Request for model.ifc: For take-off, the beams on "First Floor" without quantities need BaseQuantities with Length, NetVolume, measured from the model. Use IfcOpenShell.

First a look at what the model holds.

```python
import ifcopenshell
import ifcopenshell.util.element
import ifcopenshell.util.unit

model = ifcopenshell.open("model.ifc")
print(model.schema)
for unit_type in ("LENGTHUNIT", "AREAUNIT", "VOLUMEUNIT"):
    print(unit_type, ifcopenshell.util.unit.calculate_unit_scale(model, unit_type))
storey = next(s for s in model.by_type("IfcBuildingStorey") if s.Name == "First Floor")
beams = [e for e in ifcopenshell.util.element.get_decomposition(storey) if e.is_a("IfcBeam")]
for e in sorted(beams, key=lambda e: e.id()):
    print(e.id(), e.is_a(), e.Name, list(ifcopenshell.util.element.get_psets(e, qtos_only=True)), sep=" | ")
```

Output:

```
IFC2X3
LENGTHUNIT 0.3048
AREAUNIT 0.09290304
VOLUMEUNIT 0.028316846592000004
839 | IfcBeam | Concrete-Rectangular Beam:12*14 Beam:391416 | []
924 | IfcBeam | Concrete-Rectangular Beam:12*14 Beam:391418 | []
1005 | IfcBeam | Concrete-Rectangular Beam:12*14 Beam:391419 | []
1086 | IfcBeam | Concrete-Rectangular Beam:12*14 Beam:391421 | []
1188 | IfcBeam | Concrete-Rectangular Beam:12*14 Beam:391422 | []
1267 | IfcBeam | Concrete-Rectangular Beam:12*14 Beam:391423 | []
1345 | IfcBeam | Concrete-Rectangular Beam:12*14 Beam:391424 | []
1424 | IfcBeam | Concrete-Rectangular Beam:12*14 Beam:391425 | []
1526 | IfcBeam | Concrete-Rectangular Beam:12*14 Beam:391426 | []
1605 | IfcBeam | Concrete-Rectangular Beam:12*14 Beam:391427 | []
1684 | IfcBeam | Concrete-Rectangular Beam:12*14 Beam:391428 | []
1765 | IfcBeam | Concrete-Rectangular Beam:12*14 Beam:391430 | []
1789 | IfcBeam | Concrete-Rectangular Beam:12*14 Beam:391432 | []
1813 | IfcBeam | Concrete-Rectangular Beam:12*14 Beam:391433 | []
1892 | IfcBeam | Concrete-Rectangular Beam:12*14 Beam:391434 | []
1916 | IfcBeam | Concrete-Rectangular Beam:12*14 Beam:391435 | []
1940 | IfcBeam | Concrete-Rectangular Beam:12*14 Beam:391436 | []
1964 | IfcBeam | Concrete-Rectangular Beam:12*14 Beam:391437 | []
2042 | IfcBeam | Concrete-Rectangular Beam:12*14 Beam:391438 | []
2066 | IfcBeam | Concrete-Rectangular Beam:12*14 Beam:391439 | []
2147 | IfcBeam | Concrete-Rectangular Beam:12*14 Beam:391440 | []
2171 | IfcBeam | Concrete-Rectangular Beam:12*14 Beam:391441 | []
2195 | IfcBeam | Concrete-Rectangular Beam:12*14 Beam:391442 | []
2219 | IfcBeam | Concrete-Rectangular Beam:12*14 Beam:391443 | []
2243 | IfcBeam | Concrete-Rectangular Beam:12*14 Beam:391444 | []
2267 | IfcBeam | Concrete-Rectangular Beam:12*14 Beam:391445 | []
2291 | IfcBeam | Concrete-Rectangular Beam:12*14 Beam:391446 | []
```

```python
import ifcopenshell
import ifcopenshell.api.pset
import ifcopenshell.geom
import ifcopenshell.util.element
import ifcopenshell.util.shape
import ifcopenshell.util.unit

model = ifcopenshell.open("model.ifc")
unit_scale = ifcopenshell.util.unit.calculate_unit_scale(model)
volume_scale = ifcopenshell.util.unit.calculate_unit_scale(model, "VOLUMEUNIT")
settings = ifcopenshell.geom.settings()

storey = next(s for s in model.by_type("IfcBuildingStorey") if s.Name == "First Floor")
beams = [e for e in ifcopenshell.util.element.get_decomposition(storey) if e.is_a("IfcBeam")]

for e in sorted(beams, key=lambda e: e.id()):
    if ifcopenshell.util.element.get_psets(e, qtos_only=True, should_inherit=False):
        continue
    # Geometry comes back in metres, in the element's own axes.
    shape = ifcopenshell.geom.create_shape(settings, e)
    values = {
        "Length": ifcopenshell.util.shape.get_max_xyz(shape.geometry) / unit_scale,
        "NetVolume": ifcopenshell.util.shape.get_volume(shape.geometry) / volume_scale,
    }
    qto = ifcopenshell.api.pset.add_qto(model, product=e, name="BaseQuantities")
    ifcopenshell.api.pset.edit_qto(model, qto=qto, properties=values)
    print(e.id(), {k: round(v, 3) for k, v in values.items()})

model.write("model_rev.ifc")
```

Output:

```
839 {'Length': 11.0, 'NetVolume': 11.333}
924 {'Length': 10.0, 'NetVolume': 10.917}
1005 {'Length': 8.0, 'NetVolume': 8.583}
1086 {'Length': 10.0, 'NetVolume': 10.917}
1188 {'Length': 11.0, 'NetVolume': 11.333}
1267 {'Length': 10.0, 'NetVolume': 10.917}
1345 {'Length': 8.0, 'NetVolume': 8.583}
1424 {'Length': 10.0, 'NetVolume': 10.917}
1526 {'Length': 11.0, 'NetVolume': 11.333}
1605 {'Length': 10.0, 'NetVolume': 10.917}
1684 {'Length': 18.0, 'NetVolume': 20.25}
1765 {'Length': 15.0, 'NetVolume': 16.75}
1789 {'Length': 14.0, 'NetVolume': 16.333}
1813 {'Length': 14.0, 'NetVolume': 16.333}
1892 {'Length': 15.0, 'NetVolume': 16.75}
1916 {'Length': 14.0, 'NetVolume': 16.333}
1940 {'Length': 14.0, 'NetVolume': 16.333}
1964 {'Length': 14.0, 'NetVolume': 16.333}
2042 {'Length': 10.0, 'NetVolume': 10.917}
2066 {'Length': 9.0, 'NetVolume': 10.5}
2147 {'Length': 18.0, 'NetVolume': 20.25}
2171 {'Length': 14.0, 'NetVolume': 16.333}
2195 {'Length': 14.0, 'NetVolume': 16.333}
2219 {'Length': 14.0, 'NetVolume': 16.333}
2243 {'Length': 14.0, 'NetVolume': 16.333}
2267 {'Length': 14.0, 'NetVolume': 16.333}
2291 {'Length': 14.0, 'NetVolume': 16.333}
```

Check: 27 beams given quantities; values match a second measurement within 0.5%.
